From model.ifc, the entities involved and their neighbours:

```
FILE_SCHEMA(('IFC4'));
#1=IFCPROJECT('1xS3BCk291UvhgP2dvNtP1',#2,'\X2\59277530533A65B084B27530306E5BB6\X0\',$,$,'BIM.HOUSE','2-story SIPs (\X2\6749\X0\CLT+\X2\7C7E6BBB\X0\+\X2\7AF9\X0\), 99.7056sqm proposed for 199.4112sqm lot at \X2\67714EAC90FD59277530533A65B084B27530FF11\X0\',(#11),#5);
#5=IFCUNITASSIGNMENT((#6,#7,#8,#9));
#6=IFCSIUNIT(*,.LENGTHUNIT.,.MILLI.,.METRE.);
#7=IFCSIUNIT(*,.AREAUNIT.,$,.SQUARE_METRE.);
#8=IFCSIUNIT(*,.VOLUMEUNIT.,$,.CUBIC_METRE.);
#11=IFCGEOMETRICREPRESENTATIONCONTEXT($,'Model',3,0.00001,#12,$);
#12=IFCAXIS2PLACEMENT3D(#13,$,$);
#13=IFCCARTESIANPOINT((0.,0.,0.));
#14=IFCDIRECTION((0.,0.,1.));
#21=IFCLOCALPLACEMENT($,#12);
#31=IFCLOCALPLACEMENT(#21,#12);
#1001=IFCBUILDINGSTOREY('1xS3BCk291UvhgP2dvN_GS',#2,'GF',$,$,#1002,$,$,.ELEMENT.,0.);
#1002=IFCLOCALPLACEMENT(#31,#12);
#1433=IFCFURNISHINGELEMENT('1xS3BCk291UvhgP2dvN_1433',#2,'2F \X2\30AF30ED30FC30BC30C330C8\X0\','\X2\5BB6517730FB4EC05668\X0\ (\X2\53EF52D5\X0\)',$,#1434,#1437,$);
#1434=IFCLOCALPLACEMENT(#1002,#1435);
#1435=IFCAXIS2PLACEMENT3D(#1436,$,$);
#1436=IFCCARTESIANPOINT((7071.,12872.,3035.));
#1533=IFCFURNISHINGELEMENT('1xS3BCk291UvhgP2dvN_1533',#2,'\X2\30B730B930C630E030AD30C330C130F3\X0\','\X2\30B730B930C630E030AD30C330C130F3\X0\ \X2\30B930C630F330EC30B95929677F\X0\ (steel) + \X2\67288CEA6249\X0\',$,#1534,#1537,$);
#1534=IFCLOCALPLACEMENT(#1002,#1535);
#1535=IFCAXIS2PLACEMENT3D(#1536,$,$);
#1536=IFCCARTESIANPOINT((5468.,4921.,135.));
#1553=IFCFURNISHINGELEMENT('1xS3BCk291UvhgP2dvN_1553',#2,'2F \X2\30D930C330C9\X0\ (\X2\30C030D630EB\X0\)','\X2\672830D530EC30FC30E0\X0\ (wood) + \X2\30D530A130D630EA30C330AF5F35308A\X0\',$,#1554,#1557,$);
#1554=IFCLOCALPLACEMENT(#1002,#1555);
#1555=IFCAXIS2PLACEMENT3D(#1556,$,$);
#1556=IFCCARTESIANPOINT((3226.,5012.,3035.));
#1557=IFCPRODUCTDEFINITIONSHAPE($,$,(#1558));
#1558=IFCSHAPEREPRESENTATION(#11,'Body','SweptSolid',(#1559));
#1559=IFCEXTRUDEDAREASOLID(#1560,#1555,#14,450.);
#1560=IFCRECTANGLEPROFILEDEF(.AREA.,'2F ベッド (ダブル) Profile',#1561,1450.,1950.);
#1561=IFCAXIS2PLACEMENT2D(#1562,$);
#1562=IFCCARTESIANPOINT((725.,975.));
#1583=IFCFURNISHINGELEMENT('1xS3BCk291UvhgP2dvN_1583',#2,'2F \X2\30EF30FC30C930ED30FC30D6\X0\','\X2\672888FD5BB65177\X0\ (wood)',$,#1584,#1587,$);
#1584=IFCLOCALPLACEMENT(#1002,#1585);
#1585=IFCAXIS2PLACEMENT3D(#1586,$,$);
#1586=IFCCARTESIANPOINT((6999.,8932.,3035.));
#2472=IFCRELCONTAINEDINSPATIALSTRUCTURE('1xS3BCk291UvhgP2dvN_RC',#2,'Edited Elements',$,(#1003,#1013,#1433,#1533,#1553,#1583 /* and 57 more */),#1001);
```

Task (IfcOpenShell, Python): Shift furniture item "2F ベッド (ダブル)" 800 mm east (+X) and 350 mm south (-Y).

```python
import ifcopenshell
import ifcopenshell.api.geometry
import ifcopenshell.util.placement

model = ifcopenshell.open("model.ifc")

item = model.by_guid("1xS3BCk291UvhgP2dvN_1553")
matrix = ifcopenshell.util.placement.get_local_placement(item.ObjectPlacement)
matrix[0, 3] += 800.0
matrix[1, 3] -= 350.0
ifcopenshell.api.geometry.edit_object_placement(model, product=item, matrix=matrix, is_si=False)

print(ifcopenshell.util.placement.get_local_placement(item.ObjectPlacement).round(3) + 0.0)

model.write("model_updated.ifc")
```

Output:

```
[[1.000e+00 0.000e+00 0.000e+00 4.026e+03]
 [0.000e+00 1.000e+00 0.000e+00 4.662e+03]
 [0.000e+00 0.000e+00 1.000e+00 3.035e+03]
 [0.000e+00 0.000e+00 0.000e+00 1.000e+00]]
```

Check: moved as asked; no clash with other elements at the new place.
